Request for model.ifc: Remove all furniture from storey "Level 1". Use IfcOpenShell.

First a look at what the model holds.

```python
import ifcopenshell
import ifcopenshell.util.element

model = ifcopenshell.open("model.ifc")
print(model.schema)
storey = next(s for s in model.by_type("IfcBuildingStorey") if s.Name == "Level 1")
furniture = [e for e in ifcopenshell.util.element.get_decomposition(storey) if e.is_a("IfcFurnishingElement")]
seen = {}
for e in furniture:
    element_type = ifcopenshell.util.element.get_type(e)
    name = element_type.Name if element_type not in (None, e) else None
    seen[name] = seen.get(name, 0) + 1
for name, count in sorted(seen.items(), key=str):
    print(count, "x", name)
```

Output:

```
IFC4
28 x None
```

```python
import ifcopenshell
import ifcopenshell.api.root
import ifcopenshell.util.element

model = ifcopenshell.open("model.ifc")

storey = next(s for s in model.by_type("IfcBuildingStorey") if s.Name == "Level 1")
furniture = [e for e in ifcopenshell.util.element.get_decomposition(storey) if e.is_a("IfcFurnishingElement")]

for e in furniture:
    ifcopenshell.api.root.remove_product(model, product=e)
print(len(furniture), "removed")

model.write("model_edited.ifc")
```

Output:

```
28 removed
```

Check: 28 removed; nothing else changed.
